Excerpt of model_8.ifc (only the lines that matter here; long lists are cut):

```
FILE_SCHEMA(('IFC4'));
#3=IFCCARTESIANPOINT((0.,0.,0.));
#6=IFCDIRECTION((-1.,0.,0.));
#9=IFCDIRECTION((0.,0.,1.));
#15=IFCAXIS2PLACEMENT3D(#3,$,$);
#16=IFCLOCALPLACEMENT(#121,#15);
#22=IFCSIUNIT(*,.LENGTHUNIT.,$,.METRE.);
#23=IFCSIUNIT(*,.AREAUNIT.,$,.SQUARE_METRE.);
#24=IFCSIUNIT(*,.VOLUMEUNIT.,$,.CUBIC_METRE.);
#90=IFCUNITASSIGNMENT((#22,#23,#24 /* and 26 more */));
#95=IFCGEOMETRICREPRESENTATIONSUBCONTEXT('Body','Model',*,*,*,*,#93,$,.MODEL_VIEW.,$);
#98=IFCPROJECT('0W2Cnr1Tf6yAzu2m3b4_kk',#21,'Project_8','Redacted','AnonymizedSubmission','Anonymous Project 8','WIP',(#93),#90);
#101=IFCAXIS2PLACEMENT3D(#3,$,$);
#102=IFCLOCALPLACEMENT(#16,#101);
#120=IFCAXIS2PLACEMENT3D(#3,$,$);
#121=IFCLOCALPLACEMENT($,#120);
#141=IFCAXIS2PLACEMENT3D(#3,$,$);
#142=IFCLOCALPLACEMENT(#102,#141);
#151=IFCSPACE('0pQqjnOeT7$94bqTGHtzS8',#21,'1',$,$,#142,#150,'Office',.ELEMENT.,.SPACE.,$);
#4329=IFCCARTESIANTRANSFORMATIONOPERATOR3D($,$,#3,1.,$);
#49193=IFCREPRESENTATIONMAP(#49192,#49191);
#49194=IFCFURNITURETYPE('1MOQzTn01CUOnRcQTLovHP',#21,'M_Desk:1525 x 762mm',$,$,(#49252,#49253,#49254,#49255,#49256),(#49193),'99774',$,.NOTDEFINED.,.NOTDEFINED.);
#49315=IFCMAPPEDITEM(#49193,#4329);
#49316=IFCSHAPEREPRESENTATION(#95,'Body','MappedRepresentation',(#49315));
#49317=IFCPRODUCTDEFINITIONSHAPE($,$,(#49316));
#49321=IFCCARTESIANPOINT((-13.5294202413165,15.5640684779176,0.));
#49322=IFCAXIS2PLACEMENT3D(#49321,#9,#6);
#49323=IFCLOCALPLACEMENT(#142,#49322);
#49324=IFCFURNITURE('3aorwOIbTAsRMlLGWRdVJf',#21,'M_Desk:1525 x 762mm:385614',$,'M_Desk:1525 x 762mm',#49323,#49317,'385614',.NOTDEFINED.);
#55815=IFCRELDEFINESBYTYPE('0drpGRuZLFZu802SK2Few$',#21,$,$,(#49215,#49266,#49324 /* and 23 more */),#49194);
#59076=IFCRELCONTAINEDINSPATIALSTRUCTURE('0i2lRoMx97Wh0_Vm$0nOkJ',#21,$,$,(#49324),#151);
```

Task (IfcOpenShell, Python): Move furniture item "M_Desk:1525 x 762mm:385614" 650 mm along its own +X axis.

```python
import ifcopenshell
import ifcopenshell.api.geometry
import ifcopenshell.util.placement

model = ifcopenshell.open("model_8.ifc")

item = model.by_id(49324)
matrix = ifcopenshell.util.placement.get_local_placement(item.ObjectPlacement)
matrix[:3, 3] += matrix[:3, 0] * 0.65
ifcopenshell.api.geometry.edit_object_placement(model, product=item, matrix=matrix, is_si=False)

print(ifcopenshell.util.placement.get_local_placement(item.ObjectPlacement).round(3) + 0.0)

model.write("model_8_updated.ifc")
```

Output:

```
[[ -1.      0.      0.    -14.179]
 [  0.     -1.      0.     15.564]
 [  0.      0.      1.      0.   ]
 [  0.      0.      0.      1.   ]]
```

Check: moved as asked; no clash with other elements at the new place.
